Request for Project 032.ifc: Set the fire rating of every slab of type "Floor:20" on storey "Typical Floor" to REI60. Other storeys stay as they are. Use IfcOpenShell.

First a look at what the model holds.

```python
import ifcopenshell
import ifcopenshell.util.element

model = ifcopenshell.open("Project 032.ifc")
print(model.schema)
storey = next(s for s in model.by_type("IfcBuildingStorey") if s.Name == "Typical Floor")
slabs = [e for e in ifcopenshell.util.element.get_decomposition(storey) if e.is_a("IfcSlab")]
seen = {}
for e in slabs:
    element_type = ifcopenshell.util.element.get_type(e)
    key = (element_type.Name if element_type != e and element_type else None, ifcopenshell.util.element.get_pset(e, "Pset_SlabCommon", "FireRating"))
    seen[key] = seen.get(key, 0) + 1
for (name, value), count in sorted(seen.items(), key=str):
    print(count, "x", name, "|", value)
```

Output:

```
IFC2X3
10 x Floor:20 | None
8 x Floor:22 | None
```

```python
import ifcopenshell
import ifcopenshell.api.pset
import ifcopenshell.util.element

model = ifcopenshell.open("Project 032.ifc")

storey = next(s for s in model.by_type("IfcBuildingStorey") if s.Name == "Typical Floor")
slabs = [e for e in ifcopenshell.util.element.get_decomposition(storey) if e.is_a("IfcSlab")]

count = 0
for e in slabs:
    element_type = ifcopenshell.util.element.get_type(e)
    if element_type in (None, e) or element_type.Name != "Floor:20":
        continue
    # add_pset returns the element's existing set when there is one.
    pset = ifcopenshell.api.pset.add_pset(model, product=e, name="Pset_SlabCommon")
    ifcopenshell.api.pset.edit_pset(model, pset=pset, properties={"FireRating": "REI60"})
    count += 1

print(count, "slabs updated")

model.write("Project 032_edited.ifc")
```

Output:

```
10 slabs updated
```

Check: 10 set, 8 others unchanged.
